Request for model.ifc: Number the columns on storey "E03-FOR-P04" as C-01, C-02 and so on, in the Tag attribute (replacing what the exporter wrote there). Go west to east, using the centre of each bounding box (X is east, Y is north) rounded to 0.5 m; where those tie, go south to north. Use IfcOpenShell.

First a look at what the model holds.

```python
import ifcopenshell
import ifcopenshell.util.element
import ifcopenshell.util.placement

model = ifcopenshell.open("model.ifc")
print(model.schema)
storey = next(s for s in model.by_type("IfcBuildingStorey") if s.Name == "E03-FOR-P04")
columns = [e for e in ifcopenshell.util.element.get_decomposition(storey) if e.is_a("IfcColumn")]
for e in sorted(columns, key=lambda e: e.id()):
    origin = ifcopenshell.util.placement.get_local_placement(e.ObjectPlacement)[:3, 3]
    print(e.id(), e.Tag, e.Name, origin.round(2) + 0.0, sep=" | ")
```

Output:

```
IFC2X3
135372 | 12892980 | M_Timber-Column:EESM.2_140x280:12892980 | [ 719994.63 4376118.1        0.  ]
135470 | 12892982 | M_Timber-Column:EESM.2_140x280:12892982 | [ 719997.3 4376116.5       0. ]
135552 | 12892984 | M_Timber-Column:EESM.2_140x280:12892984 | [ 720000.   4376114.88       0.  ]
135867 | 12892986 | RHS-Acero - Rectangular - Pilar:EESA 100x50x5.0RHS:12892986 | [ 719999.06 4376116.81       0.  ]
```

```python
import ifcopenshell
import ifcopenshell.geom
import ifcopenshell.util.element
import ifcopenshell.util.shape

model = ifcopenshell.open("model.ifc")
settings = ifcopenshell.geom.settings()
settings.set("use-world-coords", True)


def centre(element):
    shape = ifcopenshell.geom.create_shape(settings, element)
    return ifcopenshell.util.shape.get_bbox_centroid(shape.geometry)


storey = next(s for s in model.by_type("IfcBuildingStorey") if s.Name == "E03-FOR-P04")
columns = [e for e in ifcopenshell.util.element.get_decomposition(storey) if e.is_a("IfcColumn")]

# Insertion points can sit at a corner or the storey origin, so sort by the geometry (in metres).
centres = {e: centre(e) for e in columns}
columns.sort(key=lambda e: (round(centres[e][0] / 0.5), centres[e][1]))

for i, e in enumerate(columns, start=1):
    number = f"C-{i:02d}"
    e.Tag = number
    print(e.id(), number)

model.write("model_rev.ifc")
```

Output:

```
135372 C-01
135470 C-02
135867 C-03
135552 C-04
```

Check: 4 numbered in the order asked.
